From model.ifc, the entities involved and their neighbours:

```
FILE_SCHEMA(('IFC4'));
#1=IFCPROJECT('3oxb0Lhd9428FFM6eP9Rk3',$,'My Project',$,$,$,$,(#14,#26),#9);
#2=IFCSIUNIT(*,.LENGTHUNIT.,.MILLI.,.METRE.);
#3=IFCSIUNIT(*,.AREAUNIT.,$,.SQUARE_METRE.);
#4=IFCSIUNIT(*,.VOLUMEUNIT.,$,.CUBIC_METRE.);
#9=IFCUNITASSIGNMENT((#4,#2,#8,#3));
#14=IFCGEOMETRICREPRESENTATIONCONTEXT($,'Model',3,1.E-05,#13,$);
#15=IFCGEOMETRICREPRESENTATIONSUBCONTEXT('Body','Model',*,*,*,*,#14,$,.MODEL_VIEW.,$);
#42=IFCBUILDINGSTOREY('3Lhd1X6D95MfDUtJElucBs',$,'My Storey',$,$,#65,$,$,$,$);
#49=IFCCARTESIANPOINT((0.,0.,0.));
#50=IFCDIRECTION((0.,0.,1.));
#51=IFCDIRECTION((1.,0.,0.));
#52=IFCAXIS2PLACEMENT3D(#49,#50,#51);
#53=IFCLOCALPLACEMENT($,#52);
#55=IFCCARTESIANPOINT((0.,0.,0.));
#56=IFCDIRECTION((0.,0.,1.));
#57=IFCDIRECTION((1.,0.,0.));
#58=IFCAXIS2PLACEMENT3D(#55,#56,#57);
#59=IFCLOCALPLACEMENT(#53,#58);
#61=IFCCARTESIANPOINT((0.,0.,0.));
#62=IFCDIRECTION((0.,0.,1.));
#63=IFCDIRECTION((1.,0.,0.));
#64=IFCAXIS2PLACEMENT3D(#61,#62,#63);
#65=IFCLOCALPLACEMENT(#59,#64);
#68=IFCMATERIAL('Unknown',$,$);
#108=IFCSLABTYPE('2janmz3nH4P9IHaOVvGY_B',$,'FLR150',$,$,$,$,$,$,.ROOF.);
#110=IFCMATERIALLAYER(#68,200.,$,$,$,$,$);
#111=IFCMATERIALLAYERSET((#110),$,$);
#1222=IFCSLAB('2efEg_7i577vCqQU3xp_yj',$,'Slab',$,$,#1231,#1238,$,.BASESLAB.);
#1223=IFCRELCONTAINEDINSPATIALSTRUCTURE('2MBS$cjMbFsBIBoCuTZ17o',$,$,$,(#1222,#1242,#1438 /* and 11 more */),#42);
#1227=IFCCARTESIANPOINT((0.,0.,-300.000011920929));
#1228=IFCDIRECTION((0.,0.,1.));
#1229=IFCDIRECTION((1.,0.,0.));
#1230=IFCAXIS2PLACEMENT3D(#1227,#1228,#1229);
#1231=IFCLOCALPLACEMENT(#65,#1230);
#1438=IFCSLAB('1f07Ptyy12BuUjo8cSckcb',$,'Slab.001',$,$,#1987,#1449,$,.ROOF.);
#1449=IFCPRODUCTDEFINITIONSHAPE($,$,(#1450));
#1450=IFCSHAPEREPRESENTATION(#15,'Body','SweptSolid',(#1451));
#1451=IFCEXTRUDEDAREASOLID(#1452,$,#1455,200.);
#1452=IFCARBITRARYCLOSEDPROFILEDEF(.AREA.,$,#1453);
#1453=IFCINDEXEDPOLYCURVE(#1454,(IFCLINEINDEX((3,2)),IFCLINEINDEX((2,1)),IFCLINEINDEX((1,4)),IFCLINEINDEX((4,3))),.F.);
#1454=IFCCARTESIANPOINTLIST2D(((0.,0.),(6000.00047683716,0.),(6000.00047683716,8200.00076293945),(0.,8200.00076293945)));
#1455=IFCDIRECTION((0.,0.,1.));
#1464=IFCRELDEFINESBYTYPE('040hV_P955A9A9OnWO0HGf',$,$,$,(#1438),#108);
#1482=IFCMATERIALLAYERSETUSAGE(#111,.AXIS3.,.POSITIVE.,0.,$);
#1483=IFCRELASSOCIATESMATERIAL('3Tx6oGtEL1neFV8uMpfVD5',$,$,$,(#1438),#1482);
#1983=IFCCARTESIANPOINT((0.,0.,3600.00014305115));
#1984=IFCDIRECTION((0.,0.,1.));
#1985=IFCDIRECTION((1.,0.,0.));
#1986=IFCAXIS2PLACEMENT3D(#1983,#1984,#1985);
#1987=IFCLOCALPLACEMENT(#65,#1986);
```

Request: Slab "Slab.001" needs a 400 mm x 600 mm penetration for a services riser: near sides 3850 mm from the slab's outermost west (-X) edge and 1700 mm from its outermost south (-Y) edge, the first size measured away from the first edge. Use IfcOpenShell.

```python
import numpy as np
import ifcopenshell
import ifcopenshell.api.feature
import ifcopenshell.api.geometry
import ifcopenshell.api.root
import ifcopenshell.geom
import ifcopenshell.util.placement
import ifcopenshell.util.representation
import ifcopenshell.util.shape
import ifcopenshell.util.unit

model = ifcopenshell.open("model.ifc")
unit_scale = ifcopenshell.util.unit.calculate_unit_scale(model)
settings = ifcopenshell.geom.settings()


def volume(element):
    """Net volume in cubic metres, openings subtracted."""
    shape = ifcopenshell.geom.create_shape(settings, element)
    return ifcopenshell.util.shape.get_volume(shape.geometry)


slab = model.by_id(1438)
before = volume(slab)

# Extent in the slab's own axes, in metres. The edges named are its -X and -Y sides.
slab_shape = ifcopenshell.geom.create_shape(settings, slab)
vertices = ifcopenshell.util.shape.get_vertices(slab_shape.geometry)
x_min, y_min, bottom = vertices.min(axis=0)
top = vertices[:, 2].max()

opening = ifcopenshell.api.root.create_entity(model, ifc_class="IfcOpeningElement", name="Services riser opening", predefined_type="OPENING")
context = ifcopenshell.util.representation.get_context(model, "Model", "Body", "MODEL_VIEW")
width, depth = 0.4, 0.6
outline = [(0.0, 0.0), (width, 0.0), (width, depth), (0.0, depth), (0.0, 0.0)]
# Overshoot both faces by 50 mm so the cut is clean.
shape = ifcopenshell.api.geometry.add_slab_representation(
    model, context=context, depth=top - bottom + 0.1, polyline=outline
)
ifcopenshell.api.geometry.assign_representation(model, product=opening, representation=shape)

matrix = ifcopenshell.util.placement.get_local_placement(slab.ObjectPlacement)
matrix[:, 3] = matrix @ np.append(np.array([x_min + 3.85, y_min + 1.7, bottom - 0.05]) / unit_scale, 1.0)
ifcopenshell.api.geometry.edit_object_placement(model, product=opening, matrix=matrix, is_si=False)
ifcopenshell.api.feature.add_feature(model, feature=opening, element=slab)

after = volume(slab)

print(f"slab volume {before:.3f} -> {after:.3f} m3")

model.write("model-out.ifc")
```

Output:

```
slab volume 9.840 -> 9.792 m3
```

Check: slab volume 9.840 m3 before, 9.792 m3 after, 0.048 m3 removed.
